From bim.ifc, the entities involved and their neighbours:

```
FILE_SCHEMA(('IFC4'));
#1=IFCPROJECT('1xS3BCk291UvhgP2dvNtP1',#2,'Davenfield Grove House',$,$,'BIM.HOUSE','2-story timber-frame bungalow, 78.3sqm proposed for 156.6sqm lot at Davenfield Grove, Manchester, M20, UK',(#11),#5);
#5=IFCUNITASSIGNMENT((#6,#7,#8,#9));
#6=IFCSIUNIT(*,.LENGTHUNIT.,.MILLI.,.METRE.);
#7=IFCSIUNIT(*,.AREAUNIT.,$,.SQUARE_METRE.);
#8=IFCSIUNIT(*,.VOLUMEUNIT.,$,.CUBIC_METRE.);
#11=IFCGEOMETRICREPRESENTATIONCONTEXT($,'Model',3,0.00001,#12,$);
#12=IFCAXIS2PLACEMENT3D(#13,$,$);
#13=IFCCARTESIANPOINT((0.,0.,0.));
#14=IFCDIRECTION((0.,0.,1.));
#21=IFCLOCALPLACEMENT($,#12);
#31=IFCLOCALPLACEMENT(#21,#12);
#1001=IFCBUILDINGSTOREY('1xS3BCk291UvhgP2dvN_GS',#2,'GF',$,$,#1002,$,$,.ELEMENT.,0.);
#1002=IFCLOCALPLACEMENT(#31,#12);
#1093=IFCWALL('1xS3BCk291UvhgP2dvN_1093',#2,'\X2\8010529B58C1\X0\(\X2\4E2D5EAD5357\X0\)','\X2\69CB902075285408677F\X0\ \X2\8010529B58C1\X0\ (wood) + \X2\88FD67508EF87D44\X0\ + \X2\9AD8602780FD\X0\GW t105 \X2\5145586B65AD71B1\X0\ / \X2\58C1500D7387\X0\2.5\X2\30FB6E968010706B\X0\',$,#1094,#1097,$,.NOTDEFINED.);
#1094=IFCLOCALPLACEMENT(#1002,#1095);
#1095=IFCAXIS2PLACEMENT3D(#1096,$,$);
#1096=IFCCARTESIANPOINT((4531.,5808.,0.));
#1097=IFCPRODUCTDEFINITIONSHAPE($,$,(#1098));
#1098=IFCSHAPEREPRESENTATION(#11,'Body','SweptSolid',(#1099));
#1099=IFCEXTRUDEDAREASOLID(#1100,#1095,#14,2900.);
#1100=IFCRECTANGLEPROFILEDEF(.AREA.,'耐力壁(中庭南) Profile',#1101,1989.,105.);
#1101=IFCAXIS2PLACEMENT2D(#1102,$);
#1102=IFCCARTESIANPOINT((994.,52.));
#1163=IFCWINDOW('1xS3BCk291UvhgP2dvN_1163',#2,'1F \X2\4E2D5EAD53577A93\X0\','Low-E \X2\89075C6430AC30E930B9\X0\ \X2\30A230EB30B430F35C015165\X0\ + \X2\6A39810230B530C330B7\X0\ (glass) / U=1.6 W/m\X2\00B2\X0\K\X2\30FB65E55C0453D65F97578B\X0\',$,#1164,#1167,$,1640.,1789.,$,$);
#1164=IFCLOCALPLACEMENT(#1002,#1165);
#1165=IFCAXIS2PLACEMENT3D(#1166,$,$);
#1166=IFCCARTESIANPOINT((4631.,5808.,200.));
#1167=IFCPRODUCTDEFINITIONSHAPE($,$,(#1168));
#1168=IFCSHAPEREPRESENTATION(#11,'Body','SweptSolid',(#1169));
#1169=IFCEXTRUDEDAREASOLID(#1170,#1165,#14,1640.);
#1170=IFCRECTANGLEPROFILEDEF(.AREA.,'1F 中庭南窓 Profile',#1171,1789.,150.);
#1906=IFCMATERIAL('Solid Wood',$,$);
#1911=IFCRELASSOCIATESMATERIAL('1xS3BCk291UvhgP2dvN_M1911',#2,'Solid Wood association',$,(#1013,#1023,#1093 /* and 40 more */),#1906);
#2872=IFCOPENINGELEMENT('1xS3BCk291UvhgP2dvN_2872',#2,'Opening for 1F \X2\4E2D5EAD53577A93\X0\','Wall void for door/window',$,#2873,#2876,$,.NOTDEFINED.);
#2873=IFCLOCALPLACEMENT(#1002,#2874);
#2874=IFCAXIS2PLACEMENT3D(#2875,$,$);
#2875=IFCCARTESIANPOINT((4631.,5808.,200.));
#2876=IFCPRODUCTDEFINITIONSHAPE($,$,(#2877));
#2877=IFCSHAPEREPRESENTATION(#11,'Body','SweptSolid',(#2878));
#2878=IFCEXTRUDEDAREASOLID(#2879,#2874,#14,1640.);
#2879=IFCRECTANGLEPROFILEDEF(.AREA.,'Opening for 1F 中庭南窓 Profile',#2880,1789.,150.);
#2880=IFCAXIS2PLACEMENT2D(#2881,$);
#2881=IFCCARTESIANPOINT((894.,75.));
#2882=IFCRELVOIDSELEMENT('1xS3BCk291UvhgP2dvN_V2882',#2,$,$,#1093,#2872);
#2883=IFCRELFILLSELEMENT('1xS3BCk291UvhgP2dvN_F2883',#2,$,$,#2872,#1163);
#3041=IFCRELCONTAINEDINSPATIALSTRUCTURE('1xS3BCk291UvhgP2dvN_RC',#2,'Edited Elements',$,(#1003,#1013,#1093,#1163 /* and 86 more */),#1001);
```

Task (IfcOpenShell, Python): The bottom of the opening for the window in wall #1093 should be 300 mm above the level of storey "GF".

```python
import numpy as np
import ifcopenshell
import ifcopenshell.api.geometry
import ifcopenshell.geom
import ifcopenshell.util.element
import ifcopenshell.util.placement
import ifcopenshell.util.shape
import ifcopenshell.util.unit

model = ifcopenshell.open("bim.ifc")
unit_scale = ifcopenshell.util.unit.calculate_unit_scale(model)

window = model.by_id(1163)
opening = window.FillsVoids[0].RelatingOpeningElement
storey = ifcopenshell.util.element.get_container(window, ifc_class="IfcBuildingStorey")
level = ifcopenshell.util.placement.get_local_placement(storey.ObjectPlacement)[2, 3]

# The opening's origin need not be at the sill, so measure its lowest point.
shape = ifcopenshell.geom.create_shape(ifcopenshell.geom.settings(), opening)
bottom = ifcopenshell.util.shape.get_shape_bottom_elevation(shape, shape.geometry) / unit_scale
dz = level + 0.3 / unit_scale - bottom

shift = np.array([0.0, 0.0, dz])
# The window is not placed relative to its opening, so move both.
for product in (opening, window):
    matrix = ifcopenshell.util.placement.get_local_placement(product.ObjectPlacement)
    matrix[:3, 3] += shift
    ifcopenshell.api.geometry.edit_object_placement(model, product=product, matrix=matrix, is_si=False)

print(f"moved by {dz * unit_scale:+.3f} m")

model.write("bim_v2.ifc")
```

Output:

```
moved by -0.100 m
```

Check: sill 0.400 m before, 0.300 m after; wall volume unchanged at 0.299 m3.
